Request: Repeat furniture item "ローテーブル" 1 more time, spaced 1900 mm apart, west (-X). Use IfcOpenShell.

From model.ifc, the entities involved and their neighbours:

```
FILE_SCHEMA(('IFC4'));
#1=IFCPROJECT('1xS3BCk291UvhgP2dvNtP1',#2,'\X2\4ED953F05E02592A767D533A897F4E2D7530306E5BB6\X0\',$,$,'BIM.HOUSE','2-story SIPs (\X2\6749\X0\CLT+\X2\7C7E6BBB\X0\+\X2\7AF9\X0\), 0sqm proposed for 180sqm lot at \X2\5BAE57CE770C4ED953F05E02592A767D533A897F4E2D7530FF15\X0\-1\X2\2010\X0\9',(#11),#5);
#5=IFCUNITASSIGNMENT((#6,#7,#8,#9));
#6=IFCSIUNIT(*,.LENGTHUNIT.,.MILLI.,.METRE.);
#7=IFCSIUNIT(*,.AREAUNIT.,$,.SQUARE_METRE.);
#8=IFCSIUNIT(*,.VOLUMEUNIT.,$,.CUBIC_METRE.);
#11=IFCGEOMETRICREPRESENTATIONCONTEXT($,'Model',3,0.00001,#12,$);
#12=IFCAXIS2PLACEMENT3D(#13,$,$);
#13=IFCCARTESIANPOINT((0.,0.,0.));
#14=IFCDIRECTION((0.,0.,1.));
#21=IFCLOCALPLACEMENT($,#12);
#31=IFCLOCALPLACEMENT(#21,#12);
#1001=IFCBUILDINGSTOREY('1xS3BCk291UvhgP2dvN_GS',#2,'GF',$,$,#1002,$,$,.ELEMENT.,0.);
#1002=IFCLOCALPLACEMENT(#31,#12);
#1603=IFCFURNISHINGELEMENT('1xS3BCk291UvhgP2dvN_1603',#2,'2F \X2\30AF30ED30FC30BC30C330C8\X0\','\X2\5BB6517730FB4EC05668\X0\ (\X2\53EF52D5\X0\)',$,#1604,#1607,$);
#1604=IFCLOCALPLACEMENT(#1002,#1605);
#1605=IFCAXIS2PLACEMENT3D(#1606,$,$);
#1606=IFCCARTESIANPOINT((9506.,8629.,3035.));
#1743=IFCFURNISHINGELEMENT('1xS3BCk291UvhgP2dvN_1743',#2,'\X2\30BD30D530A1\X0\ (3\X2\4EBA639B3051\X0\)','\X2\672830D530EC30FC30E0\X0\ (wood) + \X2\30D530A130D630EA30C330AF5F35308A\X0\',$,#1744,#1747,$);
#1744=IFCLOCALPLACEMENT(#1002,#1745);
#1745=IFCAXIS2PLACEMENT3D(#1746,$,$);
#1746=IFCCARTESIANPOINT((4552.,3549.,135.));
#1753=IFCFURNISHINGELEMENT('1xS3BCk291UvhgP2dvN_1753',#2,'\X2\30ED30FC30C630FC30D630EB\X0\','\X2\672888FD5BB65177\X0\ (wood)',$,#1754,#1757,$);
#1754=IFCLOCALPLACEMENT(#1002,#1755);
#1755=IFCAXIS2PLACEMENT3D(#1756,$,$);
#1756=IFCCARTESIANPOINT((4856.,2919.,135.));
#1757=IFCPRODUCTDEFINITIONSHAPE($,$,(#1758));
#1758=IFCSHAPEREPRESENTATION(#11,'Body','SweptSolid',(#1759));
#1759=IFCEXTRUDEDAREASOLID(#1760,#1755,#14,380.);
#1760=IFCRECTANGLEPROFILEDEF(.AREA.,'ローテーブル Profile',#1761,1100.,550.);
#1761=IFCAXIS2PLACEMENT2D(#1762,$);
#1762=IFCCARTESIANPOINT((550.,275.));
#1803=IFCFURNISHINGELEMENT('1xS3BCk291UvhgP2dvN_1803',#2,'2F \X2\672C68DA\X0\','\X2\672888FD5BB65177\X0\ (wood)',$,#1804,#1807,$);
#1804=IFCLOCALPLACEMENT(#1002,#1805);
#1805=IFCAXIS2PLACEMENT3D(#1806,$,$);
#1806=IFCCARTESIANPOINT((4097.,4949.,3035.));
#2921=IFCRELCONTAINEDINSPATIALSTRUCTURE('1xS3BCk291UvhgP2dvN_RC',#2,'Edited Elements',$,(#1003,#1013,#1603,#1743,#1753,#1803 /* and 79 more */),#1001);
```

```python
import numpy as np
import ifcopenshell
import ifcopenshell.api.geometry
import ifcopenshell.api.root
import ifcopenshell.util.element
import ifcopenshell.util.placement
import ifcopenshell.util.unit

model = ifcopenshell.open("model.ifc")
unit_scale = ifcopenshell.util.unit.calculate_unit_scale(model)


def reuse_history(source, copy):
    """copy_class also copies each property set's owner history, people and application; keep the originals."""
    for rel in copy.IsDefinedBy:
        if rel.is_a("IfcRelDefinesByProperties") and (history := rel.RelatingPropertyDefinition.OwnerHistory):
            rel.RelatingPropertyDefinition.OwnerHistory = source.OwnerHistory
            ifcopenshell.util.element.remove_deep2(model, history)


source = model.by_guid("1xS3BCk291UvhgP2dvN_1753")
base = ifcopenshell.util.placement.get_local_placement(source.ObjectPlacement)
step = np.array([-1.0, 0.0, 0.0]) * 1.9 / unit_scale

for i in range(1, 2):
    copy = ifcopenshell.api.root.copy_class(model, product=source)
    copy.Representation = ifcopenshell.util.element.copy_deep(
        model, source.Representation, exclude=["IfcGeometricRepresentationContext", "IfcRepresentationMap"]
    )
    reuse_history(source, copy)
    matrix = base.copy()
    matrix[:3, 3] += i * step
    print("added at", matrix[:3, 3].round(3) + 0.0)
    ifcopenshell.api.geometry.edit_object_placement(model, product=copy, matrix=matrix, is_si=False)

model.write("model-out.ifc")
```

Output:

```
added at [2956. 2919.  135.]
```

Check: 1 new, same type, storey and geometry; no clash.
